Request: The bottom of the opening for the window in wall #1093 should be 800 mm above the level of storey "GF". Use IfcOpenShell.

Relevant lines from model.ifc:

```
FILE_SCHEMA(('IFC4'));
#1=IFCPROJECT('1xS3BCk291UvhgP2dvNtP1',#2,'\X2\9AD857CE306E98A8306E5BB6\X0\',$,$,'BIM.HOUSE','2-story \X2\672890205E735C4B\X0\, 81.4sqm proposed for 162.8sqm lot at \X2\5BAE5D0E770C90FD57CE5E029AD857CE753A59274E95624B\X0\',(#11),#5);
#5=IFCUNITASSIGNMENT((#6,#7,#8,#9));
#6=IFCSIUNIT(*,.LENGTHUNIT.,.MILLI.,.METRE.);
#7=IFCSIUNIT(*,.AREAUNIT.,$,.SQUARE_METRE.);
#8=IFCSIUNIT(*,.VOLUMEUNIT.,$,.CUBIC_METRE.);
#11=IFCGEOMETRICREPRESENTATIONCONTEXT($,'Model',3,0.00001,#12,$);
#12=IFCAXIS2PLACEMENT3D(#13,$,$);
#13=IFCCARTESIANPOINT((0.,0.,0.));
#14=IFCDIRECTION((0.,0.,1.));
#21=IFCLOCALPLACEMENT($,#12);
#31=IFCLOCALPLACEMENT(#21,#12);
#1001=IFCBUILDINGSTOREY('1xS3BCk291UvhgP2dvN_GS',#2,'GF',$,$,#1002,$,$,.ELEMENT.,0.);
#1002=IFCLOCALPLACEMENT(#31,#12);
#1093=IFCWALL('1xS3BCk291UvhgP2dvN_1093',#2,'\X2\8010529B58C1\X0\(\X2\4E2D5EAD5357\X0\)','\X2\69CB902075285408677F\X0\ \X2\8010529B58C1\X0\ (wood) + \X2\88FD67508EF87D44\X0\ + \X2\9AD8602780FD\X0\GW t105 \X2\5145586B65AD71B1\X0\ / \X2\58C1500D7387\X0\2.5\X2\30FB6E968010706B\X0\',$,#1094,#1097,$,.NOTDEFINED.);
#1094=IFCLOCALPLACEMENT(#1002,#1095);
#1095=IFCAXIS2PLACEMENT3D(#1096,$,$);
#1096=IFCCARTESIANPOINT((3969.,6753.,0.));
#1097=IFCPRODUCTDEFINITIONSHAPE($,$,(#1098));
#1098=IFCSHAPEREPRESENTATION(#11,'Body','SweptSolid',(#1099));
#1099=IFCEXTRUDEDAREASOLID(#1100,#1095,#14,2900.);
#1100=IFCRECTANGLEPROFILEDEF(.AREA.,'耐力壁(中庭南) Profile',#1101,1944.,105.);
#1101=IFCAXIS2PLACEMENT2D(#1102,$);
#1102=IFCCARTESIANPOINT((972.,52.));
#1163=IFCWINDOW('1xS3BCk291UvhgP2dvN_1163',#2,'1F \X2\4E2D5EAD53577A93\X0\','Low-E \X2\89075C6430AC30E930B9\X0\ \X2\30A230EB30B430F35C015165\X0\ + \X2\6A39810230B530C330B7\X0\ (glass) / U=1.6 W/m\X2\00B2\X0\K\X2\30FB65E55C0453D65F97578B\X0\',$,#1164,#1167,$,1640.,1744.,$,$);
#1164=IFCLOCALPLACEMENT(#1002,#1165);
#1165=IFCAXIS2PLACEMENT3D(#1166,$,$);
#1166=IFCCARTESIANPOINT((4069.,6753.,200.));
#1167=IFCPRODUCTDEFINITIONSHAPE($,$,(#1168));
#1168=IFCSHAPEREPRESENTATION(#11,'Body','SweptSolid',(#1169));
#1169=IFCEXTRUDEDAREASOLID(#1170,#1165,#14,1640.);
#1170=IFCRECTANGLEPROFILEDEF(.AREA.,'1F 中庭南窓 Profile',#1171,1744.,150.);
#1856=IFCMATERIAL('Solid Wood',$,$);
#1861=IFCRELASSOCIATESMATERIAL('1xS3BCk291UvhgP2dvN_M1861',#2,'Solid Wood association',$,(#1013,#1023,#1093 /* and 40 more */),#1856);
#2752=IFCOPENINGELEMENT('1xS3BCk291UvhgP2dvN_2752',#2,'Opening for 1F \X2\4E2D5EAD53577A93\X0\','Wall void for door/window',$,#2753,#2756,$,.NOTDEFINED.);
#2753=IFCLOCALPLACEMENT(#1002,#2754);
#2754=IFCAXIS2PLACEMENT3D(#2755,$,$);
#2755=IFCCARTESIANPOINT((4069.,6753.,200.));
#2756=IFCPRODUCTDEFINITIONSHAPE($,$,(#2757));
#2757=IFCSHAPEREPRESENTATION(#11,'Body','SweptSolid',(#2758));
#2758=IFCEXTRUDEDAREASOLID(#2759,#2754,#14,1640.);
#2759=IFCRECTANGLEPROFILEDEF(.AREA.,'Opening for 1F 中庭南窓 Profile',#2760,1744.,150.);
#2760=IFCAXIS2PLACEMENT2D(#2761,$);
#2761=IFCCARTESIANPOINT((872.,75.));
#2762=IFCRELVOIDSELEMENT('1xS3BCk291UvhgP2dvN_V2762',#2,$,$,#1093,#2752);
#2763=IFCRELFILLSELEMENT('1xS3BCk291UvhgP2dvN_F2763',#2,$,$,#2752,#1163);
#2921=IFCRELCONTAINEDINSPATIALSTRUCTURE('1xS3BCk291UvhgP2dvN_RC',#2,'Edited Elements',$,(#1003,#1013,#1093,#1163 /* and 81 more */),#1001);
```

```python
import numpy as np
import ifcopenshell
import ifcopenshell.api.geometry
import ifcopenshell.geom
import ifcopenshell.util.element
import ifcopenshell.util.placement
import ifcopenshell.util.shape
import ifcopenshell.util.unit

model = ifcopenshell.open("model.ifc")
unit_scale = ifcopenshell.util.unit.calculate_unit_scale(model)

window = model.by_guid("1xS3BCk291UvhgP2dvN_1163")
opening = window.FillsVoids[0].RelatingOpeningElement
storey = ifcopenshell.util.element.get_container(window, ifc_class="IfcBuildingStorey")
level = ifcopenshell.util.placement.get_local_placement(storey.ObjectPlacement)[2, 3]

# The opening's origin need not be at the sill, so measure its lowest point.
shape = ifcopenshell.geom.create_shape(ifcopenshell.geom.settings(), opening)
bottom = ifcopenshell.util.shape.get_shape_bottom_elevation(shape, shape.geometry) / unit_scale
dz = level + 0.8 / unit_scale - bottom

shift = np.array([0.0, 0.0, dz])
# The window is not placed relative to its opening, so move both.
for product in (opening, window):
    matrix = ifcopenshell.util.placement.get_local_placement(product.ObjectPlacement)
    matrix[:3, 3] += shift
    ifcopenshell.api.geometry.edit_object_placement(model, product=product, matrix=matrix, is_si=False)

print(f"moved by {dz * unit_scale:+.3f} m")

model.write("model_rev.ifc")
```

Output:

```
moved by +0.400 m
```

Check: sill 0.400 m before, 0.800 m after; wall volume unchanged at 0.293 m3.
